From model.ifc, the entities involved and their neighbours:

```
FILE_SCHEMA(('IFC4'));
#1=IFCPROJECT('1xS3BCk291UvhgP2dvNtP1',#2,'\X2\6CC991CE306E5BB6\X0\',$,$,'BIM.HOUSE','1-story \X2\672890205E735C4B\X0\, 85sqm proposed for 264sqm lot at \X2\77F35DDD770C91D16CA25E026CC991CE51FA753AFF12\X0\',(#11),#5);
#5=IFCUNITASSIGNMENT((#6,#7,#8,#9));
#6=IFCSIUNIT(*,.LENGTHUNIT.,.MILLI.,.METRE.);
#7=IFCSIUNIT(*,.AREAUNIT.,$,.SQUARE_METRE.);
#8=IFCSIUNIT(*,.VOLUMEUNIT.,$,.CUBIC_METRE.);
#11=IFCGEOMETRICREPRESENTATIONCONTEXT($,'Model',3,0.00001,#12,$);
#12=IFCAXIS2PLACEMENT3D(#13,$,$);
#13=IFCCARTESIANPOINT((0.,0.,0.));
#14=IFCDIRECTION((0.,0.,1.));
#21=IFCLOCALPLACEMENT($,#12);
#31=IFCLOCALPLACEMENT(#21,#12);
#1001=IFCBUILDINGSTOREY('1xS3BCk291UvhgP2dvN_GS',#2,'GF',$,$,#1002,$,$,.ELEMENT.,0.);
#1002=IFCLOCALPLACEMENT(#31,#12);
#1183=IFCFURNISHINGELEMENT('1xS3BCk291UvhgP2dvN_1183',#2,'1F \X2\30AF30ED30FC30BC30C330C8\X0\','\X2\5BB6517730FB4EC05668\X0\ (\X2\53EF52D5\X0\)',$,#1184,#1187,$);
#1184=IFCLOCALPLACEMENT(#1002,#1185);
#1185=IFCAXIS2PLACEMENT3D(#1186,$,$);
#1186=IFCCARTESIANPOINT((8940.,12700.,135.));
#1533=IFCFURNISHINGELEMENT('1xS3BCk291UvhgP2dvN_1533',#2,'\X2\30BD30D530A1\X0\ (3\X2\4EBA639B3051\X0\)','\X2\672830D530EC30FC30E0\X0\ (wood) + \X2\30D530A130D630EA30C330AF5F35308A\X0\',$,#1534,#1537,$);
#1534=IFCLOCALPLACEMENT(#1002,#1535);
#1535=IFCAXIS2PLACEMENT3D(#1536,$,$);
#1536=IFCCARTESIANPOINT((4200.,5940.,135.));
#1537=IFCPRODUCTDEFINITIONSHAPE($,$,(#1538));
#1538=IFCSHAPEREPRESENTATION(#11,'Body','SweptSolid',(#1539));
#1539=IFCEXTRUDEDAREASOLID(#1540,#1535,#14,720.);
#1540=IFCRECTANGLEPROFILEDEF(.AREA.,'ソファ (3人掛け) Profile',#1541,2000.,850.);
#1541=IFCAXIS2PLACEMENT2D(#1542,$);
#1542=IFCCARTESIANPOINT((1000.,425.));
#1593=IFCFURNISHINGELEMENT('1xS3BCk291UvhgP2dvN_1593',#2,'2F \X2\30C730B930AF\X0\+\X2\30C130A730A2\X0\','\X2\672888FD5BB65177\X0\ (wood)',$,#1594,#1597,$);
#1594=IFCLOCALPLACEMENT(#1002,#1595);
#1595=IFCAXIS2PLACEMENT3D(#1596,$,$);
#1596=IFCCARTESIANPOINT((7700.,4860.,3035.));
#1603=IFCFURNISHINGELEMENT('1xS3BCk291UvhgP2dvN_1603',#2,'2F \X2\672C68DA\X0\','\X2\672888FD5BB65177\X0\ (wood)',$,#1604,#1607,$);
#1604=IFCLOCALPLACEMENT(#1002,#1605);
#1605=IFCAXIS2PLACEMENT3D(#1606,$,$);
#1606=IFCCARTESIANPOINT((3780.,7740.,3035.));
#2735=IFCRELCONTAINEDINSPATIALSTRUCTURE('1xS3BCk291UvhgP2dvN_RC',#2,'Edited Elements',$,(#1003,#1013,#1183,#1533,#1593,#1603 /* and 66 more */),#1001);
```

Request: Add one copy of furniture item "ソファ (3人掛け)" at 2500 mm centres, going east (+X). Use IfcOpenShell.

```python
import numpy as np
import ifcopenshell
import ifcopenshell.api.geometry
import ifcopenshell.api.root
import ifcopenshell.util.element
import ifcopenshell.util.placement
import ifcopenshell.util.unit

model = ifcopenshell.open("model.ifc")
unit_scale = ifcopenshell.util.unit.calculate_unit_scale(model)


def reuse_history(source, copy):
    """copy_class also copies each property set's owner history, people and application; keep the originals."""
    for rel in copy.IsDefinedBy:
        if rel.is_a("IfcRelDefinesByProperties") and (history := rel.RelatingPropertyDefinition.OwnerHistory):
            rel.RelatingPropertyDefinition.OwnerHistory = source.OwnerHistory
            ifcopenshell.util.element.remove_deep2(model, history)


source = model.by_id(1533)
base = ifcopenshell.util.placement.get_local_placement(source.ObjectPlacement)
step = np.array([1.0, 0.0, 0.0]) * 2.5 / unit_scale

for i in range(1, 2):
    copy = ifcopenshell.api.root.copy_class(model, product=source)
    copy.Representation = ifcopenshell.util.element.copy_deep(
        model, source.Representation, exclude=["IfcGeometricRepresentationContext", "IfcRepresentationMap"]
    )
    reuse_history(source, copy)
    matrix = base.copy()
    matrix[:3, 3] += i * step
    print("added at", matrix[:3, 3].round(3) + 0.0)
    ifcopenshell.api.geometry.edit_object_placement(model, product=copy, matrix=matrix, is_si=False)

model.write("model_updated.ifc")
```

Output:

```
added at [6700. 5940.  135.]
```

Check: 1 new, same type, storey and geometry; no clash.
